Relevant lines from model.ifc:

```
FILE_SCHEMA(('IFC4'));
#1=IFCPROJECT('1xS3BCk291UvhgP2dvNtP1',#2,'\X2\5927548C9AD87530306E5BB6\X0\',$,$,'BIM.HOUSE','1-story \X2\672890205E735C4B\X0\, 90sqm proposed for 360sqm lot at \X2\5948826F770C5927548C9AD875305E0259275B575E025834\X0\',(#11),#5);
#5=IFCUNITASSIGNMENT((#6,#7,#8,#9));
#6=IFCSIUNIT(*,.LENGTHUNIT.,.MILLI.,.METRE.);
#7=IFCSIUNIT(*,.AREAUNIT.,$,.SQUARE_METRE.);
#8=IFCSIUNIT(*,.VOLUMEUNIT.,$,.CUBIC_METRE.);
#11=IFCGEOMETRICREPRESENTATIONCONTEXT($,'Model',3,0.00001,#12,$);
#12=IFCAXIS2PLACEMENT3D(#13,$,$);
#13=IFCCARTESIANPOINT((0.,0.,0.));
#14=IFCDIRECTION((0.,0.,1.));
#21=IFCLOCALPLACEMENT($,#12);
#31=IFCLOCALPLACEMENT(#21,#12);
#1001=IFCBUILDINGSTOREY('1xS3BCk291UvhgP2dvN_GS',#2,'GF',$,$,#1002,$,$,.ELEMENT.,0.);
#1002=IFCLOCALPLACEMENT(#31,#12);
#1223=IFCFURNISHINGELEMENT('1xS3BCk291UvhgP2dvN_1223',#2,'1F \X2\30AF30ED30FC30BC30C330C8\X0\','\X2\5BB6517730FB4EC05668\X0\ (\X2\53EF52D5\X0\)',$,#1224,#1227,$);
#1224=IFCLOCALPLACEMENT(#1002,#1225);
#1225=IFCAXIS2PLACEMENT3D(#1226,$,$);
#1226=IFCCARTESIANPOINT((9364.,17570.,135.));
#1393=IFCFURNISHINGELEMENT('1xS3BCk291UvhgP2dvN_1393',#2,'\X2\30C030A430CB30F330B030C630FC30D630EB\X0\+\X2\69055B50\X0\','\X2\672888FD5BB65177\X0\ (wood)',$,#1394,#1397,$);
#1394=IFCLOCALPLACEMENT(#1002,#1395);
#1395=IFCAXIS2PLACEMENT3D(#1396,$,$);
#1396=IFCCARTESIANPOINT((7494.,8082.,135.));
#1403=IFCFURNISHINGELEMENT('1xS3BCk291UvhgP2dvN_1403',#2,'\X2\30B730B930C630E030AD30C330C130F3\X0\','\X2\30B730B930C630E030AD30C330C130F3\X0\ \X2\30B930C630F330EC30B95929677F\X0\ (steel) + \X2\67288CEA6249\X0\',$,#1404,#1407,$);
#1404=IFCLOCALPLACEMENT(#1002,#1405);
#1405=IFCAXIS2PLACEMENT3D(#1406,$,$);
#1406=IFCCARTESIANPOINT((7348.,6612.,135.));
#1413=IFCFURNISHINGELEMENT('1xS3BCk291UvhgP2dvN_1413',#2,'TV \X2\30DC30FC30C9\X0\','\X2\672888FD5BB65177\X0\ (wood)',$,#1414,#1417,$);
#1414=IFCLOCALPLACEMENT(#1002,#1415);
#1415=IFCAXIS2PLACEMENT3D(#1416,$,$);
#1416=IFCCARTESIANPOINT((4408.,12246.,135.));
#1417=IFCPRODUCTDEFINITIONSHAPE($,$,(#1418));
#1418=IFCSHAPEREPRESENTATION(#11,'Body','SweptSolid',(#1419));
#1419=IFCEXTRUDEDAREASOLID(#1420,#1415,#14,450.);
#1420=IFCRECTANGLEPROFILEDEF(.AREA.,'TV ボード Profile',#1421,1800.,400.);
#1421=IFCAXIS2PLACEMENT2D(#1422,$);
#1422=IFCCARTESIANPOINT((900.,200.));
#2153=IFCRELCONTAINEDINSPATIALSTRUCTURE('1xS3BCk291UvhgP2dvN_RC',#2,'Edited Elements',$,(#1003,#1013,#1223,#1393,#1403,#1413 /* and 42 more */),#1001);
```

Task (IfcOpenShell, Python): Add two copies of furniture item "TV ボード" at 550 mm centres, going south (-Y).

```python
import numpy as np
import ifcopenshell
import ifcopenshell.api.geometry
import ifcopenshell.api.root
import ifcopenshell.util.element
import ifcopenshell.util.placement

model = ifcopenshell.open("model.ifc")


def reuse_history(source, copy):
    """copy_class also copies each property set's owner history, people and application; keep the originals."""
    for rel in copy.IsDefinedBy:
        if rel.is_a("IfcRelDefinesByProperties") and (history := rel.RelatingPropertyDefinition.OwnerHistory):
            rel.RelatingPropertyDefinition.OwnerHistory = source.OwnerHistory
            ifcopenshell.util.element.remove_deep2(model, history)


source = model.by_guid("1xS3BCk291UvhgP2dvN_1413")
base = ifcopenshell.util.placement.get_local_placement(source.ObjectPlacement)
step = np.array([0.0, -1.0, 0.0]) * 550.0

for i in range(1, 3):
    copy = ifcopenshell.api.root.copy_class(model, product=source)
    copy.Representation = ifcopenshell.util.element.copy_deep(
        model, source.Representation, exclude=["IfcGeometricRepresentationContext", "IfcRepresentationMap"]
    )
    reuse_history(source, copy)
    matrix = base.copy()
    matrix[:3, 3] += i * step
    print("added at", matrix[:3, 3].round(3) + 0.0)
    ifcopenshell.api.geometry.edit_object_placement(model, product=copy, matrix=matrix, is_si=False)

model.write("model_edited.ifc")
```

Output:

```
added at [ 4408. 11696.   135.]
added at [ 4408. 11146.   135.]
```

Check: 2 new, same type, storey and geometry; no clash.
